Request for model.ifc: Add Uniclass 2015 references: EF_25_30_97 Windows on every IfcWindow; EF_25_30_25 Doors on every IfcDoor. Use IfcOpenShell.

First a look at what the model holds.

```python
import ifcopenshell

model = ifcopenshell.open("model.ifc")
print(model.schema)
print("classifications:", [c.Name for c in model.by_type("IfcClassification")])
for ifc_class in ("IfcDoor", "IfcRoof", "IfcStair", "IfcWall", "IfcWindow"):
    print(ifc_class, len(model.by_type(ifc_class)))
```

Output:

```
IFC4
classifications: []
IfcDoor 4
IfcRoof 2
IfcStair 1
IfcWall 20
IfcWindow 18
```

```python
import ifcopenshell
import ifcopenshell.api.classification

model = ifcopenshell.open("model.ifc")

system = ifcopenshell.api.classification.add_classification(model, classification="Uniclass 2015")

codes = {
    "IfcWindow": ("EF_25_30_97", "Windows"),
    "IfcDoor": ("EF_25_30_25", "Doors"),
}
for ifc_class, (code, name) in codes.items():
    products = model.by_type(ifc_class)
    ifcopenshell.api.classification.add_reference(
        model, products=products, classification=system, identification=code, name=name
    )
    print(code, len(products))

model.write("model_edited.ifc")
```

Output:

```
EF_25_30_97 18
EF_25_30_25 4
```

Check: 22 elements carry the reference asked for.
